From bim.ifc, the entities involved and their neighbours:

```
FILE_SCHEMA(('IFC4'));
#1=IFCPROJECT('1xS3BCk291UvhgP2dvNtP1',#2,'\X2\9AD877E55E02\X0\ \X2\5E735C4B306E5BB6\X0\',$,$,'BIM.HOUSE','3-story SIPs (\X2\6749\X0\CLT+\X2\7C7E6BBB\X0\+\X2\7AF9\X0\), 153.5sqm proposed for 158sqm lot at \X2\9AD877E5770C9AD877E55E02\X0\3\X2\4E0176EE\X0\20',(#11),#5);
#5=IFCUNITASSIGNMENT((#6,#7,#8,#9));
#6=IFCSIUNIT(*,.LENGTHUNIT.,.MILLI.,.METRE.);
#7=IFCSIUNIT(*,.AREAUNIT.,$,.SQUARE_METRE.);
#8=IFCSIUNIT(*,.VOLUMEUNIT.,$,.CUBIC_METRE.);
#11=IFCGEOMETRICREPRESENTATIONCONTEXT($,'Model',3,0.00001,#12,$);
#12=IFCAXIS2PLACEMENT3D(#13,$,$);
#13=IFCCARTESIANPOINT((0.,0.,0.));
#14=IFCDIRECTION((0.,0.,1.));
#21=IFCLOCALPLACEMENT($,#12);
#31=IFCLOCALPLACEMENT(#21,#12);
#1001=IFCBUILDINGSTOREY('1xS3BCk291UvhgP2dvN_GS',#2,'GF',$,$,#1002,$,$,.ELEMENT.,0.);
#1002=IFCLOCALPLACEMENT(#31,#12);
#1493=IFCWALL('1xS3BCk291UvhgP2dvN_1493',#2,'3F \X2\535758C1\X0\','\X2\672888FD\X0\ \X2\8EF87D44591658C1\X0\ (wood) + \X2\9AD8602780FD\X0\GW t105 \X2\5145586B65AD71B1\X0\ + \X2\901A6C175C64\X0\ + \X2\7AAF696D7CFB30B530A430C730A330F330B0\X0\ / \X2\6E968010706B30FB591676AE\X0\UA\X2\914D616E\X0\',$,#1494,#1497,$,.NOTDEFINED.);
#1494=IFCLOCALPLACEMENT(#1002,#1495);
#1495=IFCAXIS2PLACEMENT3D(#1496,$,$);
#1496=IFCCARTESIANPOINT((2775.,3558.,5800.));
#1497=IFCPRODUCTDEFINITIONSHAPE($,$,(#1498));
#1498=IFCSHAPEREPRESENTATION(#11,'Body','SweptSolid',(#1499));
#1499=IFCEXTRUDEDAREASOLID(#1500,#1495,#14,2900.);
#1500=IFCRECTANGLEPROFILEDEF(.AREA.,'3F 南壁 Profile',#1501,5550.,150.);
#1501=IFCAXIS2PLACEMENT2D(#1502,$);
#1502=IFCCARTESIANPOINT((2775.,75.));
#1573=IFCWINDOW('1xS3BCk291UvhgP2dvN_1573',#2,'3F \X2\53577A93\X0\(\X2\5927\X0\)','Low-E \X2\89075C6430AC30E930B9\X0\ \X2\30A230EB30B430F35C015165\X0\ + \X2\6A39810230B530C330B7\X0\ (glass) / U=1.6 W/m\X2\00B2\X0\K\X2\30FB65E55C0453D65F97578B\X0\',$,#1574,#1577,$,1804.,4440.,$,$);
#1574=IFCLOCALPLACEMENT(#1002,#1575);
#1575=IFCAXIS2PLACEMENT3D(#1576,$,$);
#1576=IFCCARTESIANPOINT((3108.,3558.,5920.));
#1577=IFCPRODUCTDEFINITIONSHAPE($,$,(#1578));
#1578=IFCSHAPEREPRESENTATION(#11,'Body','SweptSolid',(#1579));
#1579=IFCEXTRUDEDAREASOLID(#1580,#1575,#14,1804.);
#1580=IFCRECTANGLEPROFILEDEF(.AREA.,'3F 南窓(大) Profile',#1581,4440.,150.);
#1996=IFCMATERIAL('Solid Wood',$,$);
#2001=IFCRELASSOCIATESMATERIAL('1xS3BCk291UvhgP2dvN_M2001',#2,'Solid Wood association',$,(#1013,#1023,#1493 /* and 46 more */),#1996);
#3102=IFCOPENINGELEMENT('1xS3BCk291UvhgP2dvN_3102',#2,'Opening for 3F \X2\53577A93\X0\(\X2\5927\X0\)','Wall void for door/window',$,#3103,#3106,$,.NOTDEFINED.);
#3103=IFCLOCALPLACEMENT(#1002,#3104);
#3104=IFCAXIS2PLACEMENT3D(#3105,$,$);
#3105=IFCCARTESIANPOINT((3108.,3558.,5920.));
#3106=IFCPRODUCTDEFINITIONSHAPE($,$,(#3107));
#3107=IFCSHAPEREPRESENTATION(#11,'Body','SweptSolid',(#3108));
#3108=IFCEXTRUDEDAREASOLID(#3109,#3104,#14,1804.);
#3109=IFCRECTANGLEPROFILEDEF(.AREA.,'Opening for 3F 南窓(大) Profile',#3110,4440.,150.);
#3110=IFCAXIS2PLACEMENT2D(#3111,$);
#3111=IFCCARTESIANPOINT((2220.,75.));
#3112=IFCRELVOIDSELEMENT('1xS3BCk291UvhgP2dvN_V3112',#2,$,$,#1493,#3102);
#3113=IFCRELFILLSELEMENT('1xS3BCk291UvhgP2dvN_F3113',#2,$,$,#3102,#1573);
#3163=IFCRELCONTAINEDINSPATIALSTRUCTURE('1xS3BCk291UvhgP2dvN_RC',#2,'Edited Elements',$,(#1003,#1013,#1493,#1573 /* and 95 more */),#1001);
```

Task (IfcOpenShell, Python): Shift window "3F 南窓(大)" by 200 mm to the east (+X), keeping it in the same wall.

```python
import ifcopenshell
import ifcopenshell.api.geometry
import ifcopenshell.util.placement
import ifcopenshell.util.unit

model = ifcopenshell.open("bim.ifc")
unit_scale = ifcopenshell.util.unit.calculate_unit_scale(model)

window = model.by_id(1573)
opening = window.FillsVoids[0].RelatingOpeningElement
wall = opening.VoidsElements[0].RelatingBuildingElement

wall_matrix = ifcopenshell.util.placement.get_local_placement(wall.ObjectPlacement)
shift = wall_matrix[:3, 0] * 0.2 / unit_scale
before = ifcopenshell.util.placement.get_local_placement(window.ObjectPlacement)[:3, 3].copy()

# The window is not placed relative to its opening, so move both.
for product in (opening, window):
    matrix = ifcopenshell.util.placement.get_local_placement(product.ObjectPlacement)
    matrix[:3, 3] += shift
    ifcopenshell.api.geometry.edit_object_placement(model, product=product, matrix=matrix, is_si=False)

after = ifcopenshell.util.placement.get_local_placement(window.ObjectPlacement)[:3, 3]
print("window moved by", (after - before).round(3) + 0.0)

model.write("bim_edited.ifc")
```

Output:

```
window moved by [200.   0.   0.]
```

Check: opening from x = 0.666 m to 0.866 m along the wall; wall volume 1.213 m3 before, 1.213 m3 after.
